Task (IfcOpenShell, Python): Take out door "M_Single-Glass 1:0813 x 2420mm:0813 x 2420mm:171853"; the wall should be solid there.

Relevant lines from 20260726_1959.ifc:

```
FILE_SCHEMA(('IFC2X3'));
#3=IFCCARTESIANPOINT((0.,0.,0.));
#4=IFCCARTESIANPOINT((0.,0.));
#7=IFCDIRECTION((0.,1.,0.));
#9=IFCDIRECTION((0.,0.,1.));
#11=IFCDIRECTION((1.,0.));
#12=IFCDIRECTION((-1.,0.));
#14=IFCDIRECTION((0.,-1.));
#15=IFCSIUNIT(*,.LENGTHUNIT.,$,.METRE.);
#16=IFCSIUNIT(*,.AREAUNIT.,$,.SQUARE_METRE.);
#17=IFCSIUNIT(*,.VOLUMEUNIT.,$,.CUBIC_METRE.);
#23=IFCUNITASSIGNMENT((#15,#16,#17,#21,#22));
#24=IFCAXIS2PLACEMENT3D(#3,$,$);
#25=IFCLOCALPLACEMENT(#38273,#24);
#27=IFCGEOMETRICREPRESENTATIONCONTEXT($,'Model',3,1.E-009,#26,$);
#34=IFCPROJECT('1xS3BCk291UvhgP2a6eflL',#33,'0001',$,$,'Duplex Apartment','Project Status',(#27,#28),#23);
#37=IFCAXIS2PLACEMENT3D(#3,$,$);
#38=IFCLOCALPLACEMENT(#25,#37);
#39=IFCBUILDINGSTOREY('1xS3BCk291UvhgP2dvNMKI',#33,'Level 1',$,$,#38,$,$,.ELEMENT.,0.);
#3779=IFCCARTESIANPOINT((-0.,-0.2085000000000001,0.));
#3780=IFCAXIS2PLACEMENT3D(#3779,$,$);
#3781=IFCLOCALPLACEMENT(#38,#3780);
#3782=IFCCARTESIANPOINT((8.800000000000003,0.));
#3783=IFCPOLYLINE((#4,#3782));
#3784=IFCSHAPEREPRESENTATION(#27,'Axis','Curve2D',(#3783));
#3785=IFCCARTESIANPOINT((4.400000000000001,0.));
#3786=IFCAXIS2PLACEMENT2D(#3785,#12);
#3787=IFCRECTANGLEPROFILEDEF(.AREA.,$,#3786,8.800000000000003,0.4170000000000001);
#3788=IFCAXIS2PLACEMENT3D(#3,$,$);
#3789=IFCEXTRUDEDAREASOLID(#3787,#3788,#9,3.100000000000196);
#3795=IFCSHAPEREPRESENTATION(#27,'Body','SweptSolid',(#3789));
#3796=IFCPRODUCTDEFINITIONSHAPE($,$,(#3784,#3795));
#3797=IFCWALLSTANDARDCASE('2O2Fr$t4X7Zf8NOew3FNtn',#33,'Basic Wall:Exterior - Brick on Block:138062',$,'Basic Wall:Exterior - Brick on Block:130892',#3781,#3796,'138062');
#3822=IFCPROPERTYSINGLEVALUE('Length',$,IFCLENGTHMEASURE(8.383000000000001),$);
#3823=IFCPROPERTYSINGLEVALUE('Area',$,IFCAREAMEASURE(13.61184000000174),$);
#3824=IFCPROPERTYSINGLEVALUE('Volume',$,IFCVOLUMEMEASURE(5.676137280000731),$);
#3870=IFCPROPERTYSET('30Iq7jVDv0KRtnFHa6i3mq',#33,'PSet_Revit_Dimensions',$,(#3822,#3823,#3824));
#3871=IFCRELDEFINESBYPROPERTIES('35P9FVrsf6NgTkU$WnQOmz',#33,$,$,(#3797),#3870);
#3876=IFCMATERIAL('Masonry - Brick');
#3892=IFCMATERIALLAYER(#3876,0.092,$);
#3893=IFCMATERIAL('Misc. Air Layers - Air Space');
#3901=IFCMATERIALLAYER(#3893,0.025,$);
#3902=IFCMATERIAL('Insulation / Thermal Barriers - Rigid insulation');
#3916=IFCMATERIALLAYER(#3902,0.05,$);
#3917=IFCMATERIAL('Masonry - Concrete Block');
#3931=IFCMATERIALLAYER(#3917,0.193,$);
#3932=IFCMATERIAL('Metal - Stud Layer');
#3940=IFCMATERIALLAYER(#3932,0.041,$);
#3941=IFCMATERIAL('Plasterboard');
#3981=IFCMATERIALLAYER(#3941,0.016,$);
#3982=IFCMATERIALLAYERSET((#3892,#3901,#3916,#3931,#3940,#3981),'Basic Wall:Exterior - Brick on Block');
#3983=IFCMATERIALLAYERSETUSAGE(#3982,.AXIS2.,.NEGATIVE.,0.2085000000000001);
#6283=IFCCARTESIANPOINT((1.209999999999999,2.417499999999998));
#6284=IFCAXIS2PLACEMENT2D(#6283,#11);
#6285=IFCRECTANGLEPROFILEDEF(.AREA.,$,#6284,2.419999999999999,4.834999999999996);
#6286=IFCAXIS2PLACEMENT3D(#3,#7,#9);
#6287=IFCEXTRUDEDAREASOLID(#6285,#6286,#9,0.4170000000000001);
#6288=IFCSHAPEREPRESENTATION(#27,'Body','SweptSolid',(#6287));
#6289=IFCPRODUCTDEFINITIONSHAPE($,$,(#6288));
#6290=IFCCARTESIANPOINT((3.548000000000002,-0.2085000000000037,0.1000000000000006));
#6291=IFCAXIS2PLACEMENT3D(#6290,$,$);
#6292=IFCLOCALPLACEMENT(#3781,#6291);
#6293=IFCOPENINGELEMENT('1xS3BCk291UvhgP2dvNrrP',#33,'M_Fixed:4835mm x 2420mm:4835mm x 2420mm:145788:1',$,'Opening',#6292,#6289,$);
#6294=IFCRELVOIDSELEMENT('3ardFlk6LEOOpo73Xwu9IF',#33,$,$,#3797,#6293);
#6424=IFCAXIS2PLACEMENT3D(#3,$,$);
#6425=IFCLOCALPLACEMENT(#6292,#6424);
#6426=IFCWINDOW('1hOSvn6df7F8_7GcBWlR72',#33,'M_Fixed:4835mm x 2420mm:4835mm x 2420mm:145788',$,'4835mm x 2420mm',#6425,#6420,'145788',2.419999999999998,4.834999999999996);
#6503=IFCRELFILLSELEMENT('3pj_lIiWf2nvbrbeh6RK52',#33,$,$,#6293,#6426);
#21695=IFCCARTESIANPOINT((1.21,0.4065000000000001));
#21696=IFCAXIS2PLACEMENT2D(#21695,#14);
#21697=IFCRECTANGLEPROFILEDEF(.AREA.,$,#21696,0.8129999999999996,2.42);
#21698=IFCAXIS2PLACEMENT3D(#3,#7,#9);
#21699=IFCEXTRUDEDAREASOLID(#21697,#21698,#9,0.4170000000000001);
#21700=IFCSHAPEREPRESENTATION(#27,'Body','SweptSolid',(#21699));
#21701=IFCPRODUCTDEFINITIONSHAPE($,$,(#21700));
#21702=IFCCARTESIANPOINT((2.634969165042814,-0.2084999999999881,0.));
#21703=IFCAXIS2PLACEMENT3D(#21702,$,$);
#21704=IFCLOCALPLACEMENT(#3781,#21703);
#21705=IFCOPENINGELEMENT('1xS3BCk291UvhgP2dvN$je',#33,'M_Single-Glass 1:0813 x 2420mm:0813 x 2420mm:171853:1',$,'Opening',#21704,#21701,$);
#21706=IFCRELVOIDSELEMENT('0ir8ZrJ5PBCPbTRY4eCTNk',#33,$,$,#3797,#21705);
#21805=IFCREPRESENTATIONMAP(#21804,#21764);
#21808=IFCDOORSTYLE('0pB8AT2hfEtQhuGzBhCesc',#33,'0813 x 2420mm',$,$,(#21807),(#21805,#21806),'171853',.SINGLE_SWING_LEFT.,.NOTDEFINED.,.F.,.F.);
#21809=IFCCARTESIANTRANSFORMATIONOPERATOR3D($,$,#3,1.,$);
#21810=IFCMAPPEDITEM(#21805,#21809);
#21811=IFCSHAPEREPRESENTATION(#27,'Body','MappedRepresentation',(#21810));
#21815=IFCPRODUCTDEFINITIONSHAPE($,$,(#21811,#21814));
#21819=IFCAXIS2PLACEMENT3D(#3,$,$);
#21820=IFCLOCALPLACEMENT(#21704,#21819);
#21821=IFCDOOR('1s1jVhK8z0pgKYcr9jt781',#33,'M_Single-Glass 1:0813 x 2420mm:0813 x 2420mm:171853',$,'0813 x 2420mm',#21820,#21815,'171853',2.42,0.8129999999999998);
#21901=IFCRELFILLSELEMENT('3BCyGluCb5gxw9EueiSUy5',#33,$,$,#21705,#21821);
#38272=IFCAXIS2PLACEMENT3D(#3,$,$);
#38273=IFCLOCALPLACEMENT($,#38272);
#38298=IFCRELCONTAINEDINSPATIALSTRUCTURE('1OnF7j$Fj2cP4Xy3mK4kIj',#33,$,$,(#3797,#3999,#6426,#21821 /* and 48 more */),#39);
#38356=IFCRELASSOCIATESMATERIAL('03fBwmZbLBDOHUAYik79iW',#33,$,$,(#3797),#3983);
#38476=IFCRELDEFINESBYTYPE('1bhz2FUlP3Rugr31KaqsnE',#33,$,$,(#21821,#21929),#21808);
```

```python
import ifcopenshell
import ifcopenshell.api.feature
import ifcopenshell.api.pset
import ifcopenshell.api.root
import ifcopenshell.geom
import ifcopenshell.util.element
import ifcopenshell.util.shape
import ifcopenshell.util.unit

model = ifcopenshell.open("20260726_1959.ifc")
area_scale = ifcopenshell.util.unit.calculate_unit_scale(model, "AREAUNIT")
volume_scale = ifcopenshell.util.unit.calculate_unit_scale(model, "VOLUMEUNIT")
settings = ifcopenshell.geom.settings()


def volume(element):
    """Net volume in cubic metres, openings subtracted."""
    shape = ifcopenshell.geom.create_shape(settings, element)
    return ifcopenshell.util.shape.get_volume(shape.geometry)


door = model.by_guid("1s1jVhK8z0pgKYcr9jt781")
opening = door.FillsVoids[0].RelatingOpeningElement
wall = opening.VoidsElements[0].RelatingBuildingElement
before = volume(wall)

ifcopenshell.api.root.remove_product(model, product=door)
ifcopenshell.api.feature.remove_feature(model, feature=opening)

after = volume(wall)
thickness = 0.417  # wall thickness in metres

# Update the wall's stored quantities.
pset = model.by_id(ifcopenshell.util.element.get_pset(wall, "PSet_Revit_Dimensions", should_inherit=False)["id"])
ifcopenshell.api.pset.edit_pset(model, pset=pset, properties={
    "Area": model.create_entity("IfcAreaMeasure", after / thickness / area_scale),
    "Volume": model.create_entity("IfcVolumeMeasure", after / volume_scale),
})

print(f"wall volume {before:.3f} -> {after:.3f} m3")

model.write("20260726_1959_updated.ifc")
```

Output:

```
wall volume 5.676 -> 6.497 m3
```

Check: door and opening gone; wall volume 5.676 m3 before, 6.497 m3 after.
